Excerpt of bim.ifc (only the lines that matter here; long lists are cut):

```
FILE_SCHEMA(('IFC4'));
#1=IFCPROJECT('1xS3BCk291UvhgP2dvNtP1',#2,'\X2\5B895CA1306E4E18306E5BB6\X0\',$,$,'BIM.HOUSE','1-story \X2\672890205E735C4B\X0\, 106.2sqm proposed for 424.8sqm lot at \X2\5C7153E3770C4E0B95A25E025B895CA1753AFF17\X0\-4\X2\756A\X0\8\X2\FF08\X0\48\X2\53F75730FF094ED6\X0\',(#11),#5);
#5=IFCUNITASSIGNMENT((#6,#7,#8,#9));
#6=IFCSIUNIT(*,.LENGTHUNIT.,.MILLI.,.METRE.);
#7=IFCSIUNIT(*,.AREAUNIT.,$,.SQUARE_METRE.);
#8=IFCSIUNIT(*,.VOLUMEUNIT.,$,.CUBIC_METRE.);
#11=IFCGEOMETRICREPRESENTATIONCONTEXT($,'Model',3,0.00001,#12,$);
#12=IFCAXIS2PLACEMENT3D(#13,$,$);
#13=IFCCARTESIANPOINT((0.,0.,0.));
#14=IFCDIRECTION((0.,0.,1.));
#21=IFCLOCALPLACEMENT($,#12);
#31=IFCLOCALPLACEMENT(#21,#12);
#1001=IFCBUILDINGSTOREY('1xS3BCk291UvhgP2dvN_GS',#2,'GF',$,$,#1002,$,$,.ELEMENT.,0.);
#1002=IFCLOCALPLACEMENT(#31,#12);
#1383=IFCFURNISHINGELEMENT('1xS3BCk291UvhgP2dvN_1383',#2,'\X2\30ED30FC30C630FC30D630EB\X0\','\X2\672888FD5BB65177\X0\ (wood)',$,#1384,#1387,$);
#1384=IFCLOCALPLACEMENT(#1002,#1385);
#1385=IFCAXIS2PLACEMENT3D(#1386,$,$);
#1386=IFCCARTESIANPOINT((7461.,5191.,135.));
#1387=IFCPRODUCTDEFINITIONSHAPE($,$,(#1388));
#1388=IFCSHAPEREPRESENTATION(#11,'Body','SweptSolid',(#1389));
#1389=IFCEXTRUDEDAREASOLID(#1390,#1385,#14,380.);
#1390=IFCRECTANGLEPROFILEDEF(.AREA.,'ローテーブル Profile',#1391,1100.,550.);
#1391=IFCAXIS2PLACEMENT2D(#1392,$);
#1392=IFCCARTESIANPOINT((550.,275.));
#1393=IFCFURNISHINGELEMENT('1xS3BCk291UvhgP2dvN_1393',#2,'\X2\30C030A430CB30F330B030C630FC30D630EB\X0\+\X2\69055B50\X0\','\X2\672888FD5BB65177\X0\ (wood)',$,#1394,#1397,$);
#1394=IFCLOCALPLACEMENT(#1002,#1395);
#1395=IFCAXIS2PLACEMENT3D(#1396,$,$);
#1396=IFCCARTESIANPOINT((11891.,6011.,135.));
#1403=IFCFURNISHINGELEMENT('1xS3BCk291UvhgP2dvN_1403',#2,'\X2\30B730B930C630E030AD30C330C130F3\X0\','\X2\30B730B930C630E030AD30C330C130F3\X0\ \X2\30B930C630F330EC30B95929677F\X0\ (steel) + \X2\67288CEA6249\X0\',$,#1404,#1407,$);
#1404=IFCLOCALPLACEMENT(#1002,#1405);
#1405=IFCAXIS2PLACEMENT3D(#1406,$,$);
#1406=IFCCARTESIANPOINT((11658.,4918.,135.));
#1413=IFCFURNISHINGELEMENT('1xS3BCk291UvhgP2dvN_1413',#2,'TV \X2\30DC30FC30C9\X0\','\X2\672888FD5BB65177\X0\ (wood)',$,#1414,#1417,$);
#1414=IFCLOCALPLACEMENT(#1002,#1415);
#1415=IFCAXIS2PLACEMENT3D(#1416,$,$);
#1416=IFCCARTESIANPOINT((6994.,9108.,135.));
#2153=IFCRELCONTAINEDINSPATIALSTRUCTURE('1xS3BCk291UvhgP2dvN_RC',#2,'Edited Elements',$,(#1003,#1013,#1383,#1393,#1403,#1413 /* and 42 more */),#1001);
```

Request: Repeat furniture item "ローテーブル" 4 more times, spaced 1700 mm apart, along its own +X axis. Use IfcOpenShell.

```python
import ifcopenshell
import ifcopenshell.api.geometry
import ifcopenshell.api.root
import ifcopenshell.util.element
import ifcopenshell.util.placement
import ifcopenshell.util.unit

model = ifcopenshell.open("bim.ifc")
unit_scale = ifcopenshell.util.unit.calculate_unit_scale(model)


def reuse_history(source, copy):
    """copy_class also copies each property set's owner history, people and application; keep the originals."""
    for rel in copy.IsDefinedBy:
        if rel.is_a("IfcRelDefinesByProperties") and (history := rel.RelatingPropertyDefinition.OwnerHistory):
            rel.RelatingPropertyDefinition.OwnerHistory = source.OwnerHistory
            ifcopenshell.util.element.remove_deep2(model, history)


source = model.by_guid("1xS3BCk291UvhgP2dvN_1383")
base = ifcopenshell.util.placement.get_local_placement(source.ObjectPlacement)
step = base[:3, 0] * 1.7 / unit_scale

for i in range(1, 5):
    copy = ifcopenshell.api.root.copy_class(model, product=source)
    copy.Representation = ifcopenshell.util.element.copy_deep(
        model, source.Representation, exclude=["IfcGeometricRepresentationContext", "IfcRepresentationMap"]
    )
    reuse_history(source, copy)
    matrix = base.copy()
    matrix[:3, 3] += i * step
    print("added at", matrix[:3, 3].round(3) + 0.0)
    ifcopenshell.api.geometry.edit_object_placement(model, product=copy, matrix=matrix, is_si=False)

model.write("bim_edited.ifc")
```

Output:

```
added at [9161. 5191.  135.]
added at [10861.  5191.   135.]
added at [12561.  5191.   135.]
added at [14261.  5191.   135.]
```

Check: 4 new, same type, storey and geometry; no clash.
